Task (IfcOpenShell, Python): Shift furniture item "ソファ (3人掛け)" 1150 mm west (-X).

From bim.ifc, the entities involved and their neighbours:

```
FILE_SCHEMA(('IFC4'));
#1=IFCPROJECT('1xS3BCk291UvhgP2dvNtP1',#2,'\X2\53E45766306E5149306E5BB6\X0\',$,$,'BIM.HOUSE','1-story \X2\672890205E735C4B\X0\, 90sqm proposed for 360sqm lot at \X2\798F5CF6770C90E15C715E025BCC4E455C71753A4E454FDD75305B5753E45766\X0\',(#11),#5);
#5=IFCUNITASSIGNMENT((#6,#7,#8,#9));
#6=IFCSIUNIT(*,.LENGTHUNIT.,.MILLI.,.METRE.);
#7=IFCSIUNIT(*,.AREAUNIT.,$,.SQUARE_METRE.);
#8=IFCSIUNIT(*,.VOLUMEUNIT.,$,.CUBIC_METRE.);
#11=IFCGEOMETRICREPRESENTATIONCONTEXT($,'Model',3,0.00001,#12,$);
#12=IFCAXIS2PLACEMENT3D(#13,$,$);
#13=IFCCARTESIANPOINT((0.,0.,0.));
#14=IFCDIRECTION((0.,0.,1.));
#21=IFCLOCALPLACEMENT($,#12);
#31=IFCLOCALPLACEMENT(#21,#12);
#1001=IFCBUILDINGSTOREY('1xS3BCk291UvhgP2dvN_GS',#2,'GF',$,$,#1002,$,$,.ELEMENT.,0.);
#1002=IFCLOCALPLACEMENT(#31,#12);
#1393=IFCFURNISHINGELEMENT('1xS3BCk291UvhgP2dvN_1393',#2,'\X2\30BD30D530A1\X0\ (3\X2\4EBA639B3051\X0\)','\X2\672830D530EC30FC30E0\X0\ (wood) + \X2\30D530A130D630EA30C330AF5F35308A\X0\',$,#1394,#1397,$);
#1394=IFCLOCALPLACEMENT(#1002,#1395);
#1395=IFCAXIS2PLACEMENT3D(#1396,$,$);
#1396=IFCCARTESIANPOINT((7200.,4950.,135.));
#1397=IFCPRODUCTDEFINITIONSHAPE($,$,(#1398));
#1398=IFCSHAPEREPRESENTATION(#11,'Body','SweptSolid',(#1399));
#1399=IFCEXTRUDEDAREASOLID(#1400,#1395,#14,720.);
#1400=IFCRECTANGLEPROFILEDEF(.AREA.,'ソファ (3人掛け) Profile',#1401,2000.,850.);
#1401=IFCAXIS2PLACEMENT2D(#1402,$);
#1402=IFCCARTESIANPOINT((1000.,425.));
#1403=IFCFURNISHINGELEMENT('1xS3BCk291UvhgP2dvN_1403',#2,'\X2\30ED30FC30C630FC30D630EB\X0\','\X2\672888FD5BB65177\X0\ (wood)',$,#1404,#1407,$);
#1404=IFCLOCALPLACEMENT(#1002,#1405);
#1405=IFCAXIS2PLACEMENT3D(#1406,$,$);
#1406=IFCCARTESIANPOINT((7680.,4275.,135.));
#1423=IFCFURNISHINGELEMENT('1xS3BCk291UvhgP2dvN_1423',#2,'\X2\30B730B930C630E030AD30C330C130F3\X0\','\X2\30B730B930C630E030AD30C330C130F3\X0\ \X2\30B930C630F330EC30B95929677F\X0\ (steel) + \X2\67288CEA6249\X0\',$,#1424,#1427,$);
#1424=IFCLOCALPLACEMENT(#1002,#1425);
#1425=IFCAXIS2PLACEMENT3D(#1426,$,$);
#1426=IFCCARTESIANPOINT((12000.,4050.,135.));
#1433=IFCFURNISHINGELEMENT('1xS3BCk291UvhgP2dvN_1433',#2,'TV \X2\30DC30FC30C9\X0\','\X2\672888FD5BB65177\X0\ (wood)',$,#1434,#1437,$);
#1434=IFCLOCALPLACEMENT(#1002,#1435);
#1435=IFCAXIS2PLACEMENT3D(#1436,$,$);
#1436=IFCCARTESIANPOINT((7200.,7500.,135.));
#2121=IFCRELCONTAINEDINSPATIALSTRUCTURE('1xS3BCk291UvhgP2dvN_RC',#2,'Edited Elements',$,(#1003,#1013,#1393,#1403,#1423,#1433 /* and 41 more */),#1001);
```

```python
import ifcopenshell
import ifcopenshell.api.geometry
import ifcopenshell.util.placement

model = ifcopenshell.open("bim.ifc")

item = model.by_guid("1xS3BCk291UvhgP2dvN_1393")
matrix = ifcopenshell.util.placement.get_local_placement(item.ObjectPlacement)
matrix[0, 3] -= 1150.0
ifcopenshell.api.geometry.edit_object_placement(model, product=item, matrix=matrix, is_si=False)

print(ifcopenshell.util.placement.get_local_placement(item.ObjectPlacement).round(3) + 0.0)

model.write("bim_v2.ifc")
```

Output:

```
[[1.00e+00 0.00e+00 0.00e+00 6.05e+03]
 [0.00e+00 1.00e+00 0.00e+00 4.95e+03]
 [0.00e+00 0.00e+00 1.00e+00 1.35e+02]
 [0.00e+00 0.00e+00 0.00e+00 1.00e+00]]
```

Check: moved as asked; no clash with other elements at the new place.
